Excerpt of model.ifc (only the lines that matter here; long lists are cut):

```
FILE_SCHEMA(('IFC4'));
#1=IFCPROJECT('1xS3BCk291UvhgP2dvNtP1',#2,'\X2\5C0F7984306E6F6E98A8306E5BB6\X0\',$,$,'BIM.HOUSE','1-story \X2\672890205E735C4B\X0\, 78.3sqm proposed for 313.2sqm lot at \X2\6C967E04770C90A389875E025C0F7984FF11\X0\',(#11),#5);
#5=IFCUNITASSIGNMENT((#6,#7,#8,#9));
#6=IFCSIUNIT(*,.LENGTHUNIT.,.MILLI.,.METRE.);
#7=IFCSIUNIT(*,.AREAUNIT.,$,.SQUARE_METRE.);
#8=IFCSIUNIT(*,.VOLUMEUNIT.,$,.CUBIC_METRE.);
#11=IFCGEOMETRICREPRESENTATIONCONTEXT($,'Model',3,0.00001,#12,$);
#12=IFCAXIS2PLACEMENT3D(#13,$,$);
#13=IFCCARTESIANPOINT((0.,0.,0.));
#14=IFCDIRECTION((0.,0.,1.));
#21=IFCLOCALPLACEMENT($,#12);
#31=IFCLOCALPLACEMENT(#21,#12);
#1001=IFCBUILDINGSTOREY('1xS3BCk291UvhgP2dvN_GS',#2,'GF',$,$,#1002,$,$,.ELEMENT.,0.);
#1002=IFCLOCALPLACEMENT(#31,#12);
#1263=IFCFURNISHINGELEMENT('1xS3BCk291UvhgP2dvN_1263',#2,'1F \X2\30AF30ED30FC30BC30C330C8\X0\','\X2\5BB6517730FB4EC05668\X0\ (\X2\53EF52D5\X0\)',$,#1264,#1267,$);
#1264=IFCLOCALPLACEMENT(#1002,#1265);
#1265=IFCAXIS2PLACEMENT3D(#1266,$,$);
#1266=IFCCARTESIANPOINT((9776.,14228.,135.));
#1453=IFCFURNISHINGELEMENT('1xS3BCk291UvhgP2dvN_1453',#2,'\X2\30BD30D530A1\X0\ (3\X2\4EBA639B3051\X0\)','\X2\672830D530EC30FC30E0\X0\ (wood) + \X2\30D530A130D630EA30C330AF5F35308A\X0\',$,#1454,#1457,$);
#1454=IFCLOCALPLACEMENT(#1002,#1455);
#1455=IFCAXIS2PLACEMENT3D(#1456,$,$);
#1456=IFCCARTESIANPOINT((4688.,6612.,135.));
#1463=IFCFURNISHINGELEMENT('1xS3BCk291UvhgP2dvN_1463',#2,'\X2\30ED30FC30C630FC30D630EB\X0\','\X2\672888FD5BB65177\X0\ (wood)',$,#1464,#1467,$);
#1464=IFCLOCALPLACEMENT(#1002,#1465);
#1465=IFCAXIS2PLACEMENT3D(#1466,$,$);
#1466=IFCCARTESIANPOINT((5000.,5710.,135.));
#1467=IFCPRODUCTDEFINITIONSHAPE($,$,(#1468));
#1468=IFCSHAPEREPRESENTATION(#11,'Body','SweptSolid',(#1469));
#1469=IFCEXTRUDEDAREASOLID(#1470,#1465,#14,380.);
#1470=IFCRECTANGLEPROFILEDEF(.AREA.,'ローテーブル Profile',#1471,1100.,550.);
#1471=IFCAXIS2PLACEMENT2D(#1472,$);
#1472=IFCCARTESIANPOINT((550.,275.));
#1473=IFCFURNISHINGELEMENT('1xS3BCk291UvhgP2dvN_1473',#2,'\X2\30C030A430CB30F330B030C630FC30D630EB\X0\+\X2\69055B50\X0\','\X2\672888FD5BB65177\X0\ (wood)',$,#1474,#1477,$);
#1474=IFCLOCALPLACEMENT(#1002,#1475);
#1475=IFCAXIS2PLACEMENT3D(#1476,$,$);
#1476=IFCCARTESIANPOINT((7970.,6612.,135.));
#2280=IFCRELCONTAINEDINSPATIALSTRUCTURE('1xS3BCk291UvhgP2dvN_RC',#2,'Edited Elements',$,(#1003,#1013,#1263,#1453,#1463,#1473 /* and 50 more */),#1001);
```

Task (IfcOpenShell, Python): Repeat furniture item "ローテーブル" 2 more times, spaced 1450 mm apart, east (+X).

```python
import numpy as np
import ifcopenshell
import ifcopenshell.api.geometry
import ifcopenshell.api.root
import ifcopenshell.util.element
import ifcopenshell.util.placement
import ifcopenshell.util.unit

model = ifcopenshell.open("model.ifc")
unit_scale = ifcopenshell.util.unit.calculate_unit_scale(model)


def reuse_history(source, copy):
    """copy_class also copies each property set's owner history, people and application; keep the originals."""
    for rel in copy.IsDefinedBy:
        if rel.is_a("IfcRelDefinesByProperties") and (history := rel.RelatingPropertyDefinition.OwnerHistory):
            rel.RelatingPropertyDefinition.OwnerHistory = source.OwnerHistory
            ifcopenshell.util.element.remove_deep2(model, history)


source = model.by_guid("1xS3BCk291UvhgP2dvN_1463")
base = ifcopenshell.util.placement.get_local_placement(source.ObjectPlacement)
step = np.array([1.0, 0.0, 0.0]) * 1.45 / unit_scale

for i in range(1, 3):
    copy = ifcopenshell.api.root.copy_class(model, product=source)
    copy.Representation = ifcopenshell.util.element.copy_deep(
        model, source.Representation, exclude=["IfcGeometricRepresentationContext", "IfcRepresentationMap"]
    )
    reuse_history(source, copy)
    matrix = base.copy()
    matrix[:3, 3] += i * step
    print("added at", matrix[:3, 3].round(3) + 0.0)
    ifcopenshell.api.geometry.edit_object_placement(model, product=copy, matrix=matrix, is_si=False)

model.write("model_rev.ifc")
```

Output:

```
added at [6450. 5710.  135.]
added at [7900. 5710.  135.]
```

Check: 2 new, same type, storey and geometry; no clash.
